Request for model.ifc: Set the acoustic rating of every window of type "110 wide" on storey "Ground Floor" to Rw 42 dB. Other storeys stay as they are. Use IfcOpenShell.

First a look at what the model holds.

```python
import ifcopenshell
import ifcopenshell.util.element

model = ifcopenshell.open("model.ifc")
print(model.schema)
storey = next(s for s in model.by_type("IfcBuildingStorey") if s.Name == "Ground Floor")
windows = [e for e in ifcopenshell.util.element.get_decomposition(storey) if e.is_a("IfcWindow")]
seen = {}
for e in windows:
    element_type = ifcopenshell.util.element.get_type(e)
    key = (element_type.Name if element_type != e and element_type else None, ifcopenshell.util.element.get_pset(e, "Pset_WindowCommon", "AcousticRating"))
    seen[key] = seen.get(key, 0) + 1
for (name, value), count in sorted(seen.items(), key=str):
    print(count, "x", name, "|", value)
```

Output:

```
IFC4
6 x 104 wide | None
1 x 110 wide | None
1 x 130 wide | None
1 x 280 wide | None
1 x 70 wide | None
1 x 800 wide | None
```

```python
import ifcopenshell
import ifcopenshell.api.pset
import ifcopenshell.util.element

model = ifcopenshell.open("model.ifc")

storey = next(s for s in model.by_type("IfcBuildingStorey") if s.Name == "Ground Floor")
windows = [e for e in ifcopenshell.util.element.get_decomposition(storey) if e.is_a("IfcWindow")]

count = 0
for e in windows:
    element_type = ifcopenshell.util.element.get_type(e)
    if element_type in (None, e) or element_type.Name != "110 wide":
        continue
    # add_pset returns the element's existing set when there is one.
    pset = ifcopenshell.api.pset.add_pset(model, product=e, name="Pset_WindowCommon")
    ifcopenshell.api.pset.edit_pset(model, pset=pset, properties={"AcousticRating": "Rw 42 dB"})
    count += 1

print(count, "windows updated")

model.write("model_rev.ifc")
```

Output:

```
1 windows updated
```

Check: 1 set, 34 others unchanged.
